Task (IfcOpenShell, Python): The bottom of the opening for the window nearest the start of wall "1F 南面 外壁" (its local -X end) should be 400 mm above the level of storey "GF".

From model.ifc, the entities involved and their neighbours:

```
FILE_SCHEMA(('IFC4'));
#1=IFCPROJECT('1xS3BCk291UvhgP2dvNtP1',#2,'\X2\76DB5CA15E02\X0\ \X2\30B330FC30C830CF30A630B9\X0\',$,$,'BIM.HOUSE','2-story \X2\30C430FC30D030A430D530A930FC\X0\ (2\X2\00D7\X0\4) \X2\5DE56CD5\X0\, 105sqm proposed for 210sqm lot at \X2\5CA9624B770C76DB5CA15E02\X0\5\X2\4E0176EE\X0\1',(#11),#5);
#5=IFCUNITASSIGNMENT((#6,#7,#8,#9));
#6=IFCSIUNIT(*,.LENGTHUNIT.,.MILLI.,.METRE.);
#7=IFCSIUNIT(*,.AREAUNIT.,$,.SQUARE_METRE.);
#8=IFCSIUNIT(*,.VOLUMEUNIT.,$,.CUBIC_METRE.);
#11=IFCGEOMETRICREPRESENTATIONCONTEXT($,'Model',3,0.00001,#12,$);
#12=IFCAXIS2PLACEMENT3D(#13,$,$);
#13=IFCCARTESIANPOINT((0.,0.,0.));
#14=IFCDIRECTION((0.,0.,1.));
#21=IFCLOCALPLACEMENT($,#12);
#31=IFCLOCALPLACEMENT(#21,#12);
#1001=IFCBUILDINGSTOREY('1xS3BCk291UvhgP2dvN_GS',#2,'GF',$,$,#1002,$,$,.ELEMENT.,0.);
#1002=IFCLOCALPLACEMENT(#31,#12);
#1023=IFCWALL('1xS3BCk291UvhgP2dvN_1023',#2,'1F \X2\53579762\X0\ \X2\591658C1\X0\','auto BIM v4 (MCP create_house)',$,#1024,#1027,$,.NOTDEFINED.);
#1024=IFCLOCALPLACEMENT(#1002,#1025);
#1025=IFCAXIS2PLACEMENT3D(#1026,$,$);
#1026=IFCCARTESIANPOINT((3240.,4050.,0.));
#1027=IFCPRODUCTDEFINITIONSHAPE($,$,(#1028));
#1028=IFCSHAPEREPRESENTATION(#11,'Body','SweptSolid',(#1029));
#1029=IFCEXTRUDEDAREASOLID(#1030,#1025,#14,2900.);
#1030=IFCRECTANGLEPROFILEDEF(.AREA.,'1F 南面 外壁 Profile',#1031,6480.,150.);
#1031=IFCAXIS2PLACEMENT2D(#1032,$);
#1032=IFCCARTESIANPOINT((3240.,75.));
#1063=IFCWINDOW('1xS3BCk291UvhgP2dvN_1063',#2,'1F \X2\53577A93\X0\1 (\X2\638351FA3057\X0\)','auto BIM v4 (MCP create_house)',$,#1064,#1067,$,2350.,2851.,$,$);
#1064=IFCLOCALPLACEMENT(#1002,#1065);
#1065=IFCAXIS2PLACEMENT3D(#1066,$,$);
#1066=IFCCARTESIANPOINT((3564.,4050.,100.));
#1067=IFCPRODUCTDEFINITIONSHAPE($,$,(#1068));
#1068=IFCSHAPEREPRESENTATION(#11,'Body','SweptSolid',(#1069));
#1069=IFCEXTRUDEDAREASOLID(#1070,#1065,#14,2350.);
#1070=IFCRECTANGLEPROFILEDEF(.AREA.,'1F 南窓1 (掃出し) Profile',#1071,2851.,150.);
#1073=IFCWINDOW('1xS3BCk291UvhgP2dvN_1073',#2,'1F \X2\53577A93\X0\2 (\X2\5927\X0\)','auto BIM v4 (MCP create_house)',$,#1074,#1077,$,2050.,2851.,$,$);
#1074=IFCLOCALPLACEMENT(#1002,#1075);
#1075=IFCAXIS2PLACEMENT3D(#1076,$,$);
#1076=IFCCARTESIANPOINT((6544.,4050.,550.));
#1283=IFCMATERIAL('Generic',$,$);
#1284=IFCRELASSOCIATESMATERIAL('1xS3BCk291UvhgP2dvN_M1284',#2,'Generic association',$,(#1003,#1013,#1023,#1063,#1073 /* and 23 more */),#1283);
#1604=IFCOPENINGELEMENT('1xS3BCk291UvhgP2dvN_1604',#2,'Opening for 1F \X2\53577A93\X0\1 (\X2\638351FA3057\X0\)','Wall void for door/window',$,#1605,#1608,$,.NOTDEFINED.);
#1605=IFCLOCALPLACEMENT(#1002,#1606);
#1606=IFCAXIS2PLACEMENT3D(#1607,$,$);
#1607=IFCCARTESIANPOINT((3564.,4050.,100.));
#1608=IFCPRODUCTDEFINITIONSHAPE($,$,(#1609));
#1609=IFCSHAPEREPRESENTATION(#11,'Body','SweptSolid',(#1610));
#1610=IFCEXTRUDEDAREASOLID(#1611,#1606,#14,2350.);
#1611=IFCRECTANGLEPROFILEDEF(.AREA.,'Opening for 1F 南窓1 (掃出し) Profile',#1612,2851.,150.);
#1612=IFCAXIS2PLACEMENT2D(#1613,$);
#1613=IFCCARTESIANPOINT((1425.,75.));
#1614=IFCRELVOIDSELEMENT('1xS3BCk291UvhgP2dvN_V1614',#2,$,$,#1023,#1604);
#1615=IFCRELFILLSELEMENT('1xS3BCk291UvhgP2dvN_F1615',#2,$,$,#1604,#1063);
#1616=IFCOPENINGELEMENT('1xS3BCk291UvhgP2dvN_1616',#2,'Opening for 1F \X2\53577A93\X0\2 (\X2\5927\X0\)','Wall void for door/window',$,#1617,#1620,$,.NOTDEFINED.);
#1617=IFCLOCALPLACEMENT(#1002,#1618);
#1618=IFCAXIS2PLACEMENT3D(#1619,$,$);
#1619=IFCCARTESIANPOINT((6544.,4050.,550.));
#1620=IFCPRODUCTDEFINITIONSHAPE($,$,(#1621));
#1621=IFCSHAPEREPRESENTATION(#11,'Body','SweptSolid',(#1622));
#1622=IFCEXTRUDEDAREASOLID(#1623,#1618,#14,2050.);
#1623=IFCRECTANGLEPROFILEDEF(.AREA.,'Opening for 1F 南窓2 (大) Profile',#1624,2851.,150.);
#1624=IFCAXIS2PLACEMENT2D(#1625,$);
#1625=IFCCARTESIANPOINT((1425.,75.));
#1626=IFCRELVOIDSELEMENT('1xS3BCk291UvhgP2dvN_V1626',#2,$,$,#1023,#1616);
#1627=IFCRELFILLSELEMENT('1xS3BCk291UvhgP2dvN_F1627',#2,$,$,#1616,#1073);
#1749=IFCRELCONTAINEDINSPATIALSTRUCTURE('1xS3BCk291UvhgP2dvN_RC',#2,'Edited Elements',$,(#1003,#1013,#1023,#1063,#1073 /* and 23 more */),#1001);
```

```python
import numpy as np
import ifcopenshell
import ifcopenshell.api.geometry
import ifcopenshell.geom
import ifcopenshell.util.element
import ifcopenshell.util.placement
import ifcopenshell.util.shape
import ifcopenshell.util.unit

model = ifcopenshell.open("model.ifc")
unit_scale = ifcopenshell.util.unit.calculate_unit_scale(model)

window = model.by_guid("1xS3BCk291UvhgP2dvN_1063")
opening = window.FillsVoids[0].RelatingOpeningElement
storey = ifcopenshell.util.element.get_container(window, ifc_class="IfcBuildingStorey")
level = ifcopenshell.util.placement.get_local_placement(storey.ObjectPlacement)[2, 3]

# The opening's origin need not be at the sill, so measure its lowest point.
shape = ifcopenshell.geom.create_shape(ifcopenshell.geom.settings(), opening)
bottom = ifcopenshell.util.shape.get_shape_bottom_elevation(shape, shape.geometry) / unit_scale
dz = level + 0.4 / unit_scale - bottom

shift = np.array([0.0, 0.0, dz])
# The window is not placed relative to its opening, so move both.
for product in (opening, window):
    matrix = ifcopenshell.util.placement.get_local_placement(product.ObjectPlacement)
    matrix[:3, 3] += shift
    ifcopenshell.api.geometry.edit_object_placement(model, product=product, matrix=matrix, is_si=False)

print(f"moved by {dz * unit_scale:+.3f} m")

model.write("model_rev.ifc")
```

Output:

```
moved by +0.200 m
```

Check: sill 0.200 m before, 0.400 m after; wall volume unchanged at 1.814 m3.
